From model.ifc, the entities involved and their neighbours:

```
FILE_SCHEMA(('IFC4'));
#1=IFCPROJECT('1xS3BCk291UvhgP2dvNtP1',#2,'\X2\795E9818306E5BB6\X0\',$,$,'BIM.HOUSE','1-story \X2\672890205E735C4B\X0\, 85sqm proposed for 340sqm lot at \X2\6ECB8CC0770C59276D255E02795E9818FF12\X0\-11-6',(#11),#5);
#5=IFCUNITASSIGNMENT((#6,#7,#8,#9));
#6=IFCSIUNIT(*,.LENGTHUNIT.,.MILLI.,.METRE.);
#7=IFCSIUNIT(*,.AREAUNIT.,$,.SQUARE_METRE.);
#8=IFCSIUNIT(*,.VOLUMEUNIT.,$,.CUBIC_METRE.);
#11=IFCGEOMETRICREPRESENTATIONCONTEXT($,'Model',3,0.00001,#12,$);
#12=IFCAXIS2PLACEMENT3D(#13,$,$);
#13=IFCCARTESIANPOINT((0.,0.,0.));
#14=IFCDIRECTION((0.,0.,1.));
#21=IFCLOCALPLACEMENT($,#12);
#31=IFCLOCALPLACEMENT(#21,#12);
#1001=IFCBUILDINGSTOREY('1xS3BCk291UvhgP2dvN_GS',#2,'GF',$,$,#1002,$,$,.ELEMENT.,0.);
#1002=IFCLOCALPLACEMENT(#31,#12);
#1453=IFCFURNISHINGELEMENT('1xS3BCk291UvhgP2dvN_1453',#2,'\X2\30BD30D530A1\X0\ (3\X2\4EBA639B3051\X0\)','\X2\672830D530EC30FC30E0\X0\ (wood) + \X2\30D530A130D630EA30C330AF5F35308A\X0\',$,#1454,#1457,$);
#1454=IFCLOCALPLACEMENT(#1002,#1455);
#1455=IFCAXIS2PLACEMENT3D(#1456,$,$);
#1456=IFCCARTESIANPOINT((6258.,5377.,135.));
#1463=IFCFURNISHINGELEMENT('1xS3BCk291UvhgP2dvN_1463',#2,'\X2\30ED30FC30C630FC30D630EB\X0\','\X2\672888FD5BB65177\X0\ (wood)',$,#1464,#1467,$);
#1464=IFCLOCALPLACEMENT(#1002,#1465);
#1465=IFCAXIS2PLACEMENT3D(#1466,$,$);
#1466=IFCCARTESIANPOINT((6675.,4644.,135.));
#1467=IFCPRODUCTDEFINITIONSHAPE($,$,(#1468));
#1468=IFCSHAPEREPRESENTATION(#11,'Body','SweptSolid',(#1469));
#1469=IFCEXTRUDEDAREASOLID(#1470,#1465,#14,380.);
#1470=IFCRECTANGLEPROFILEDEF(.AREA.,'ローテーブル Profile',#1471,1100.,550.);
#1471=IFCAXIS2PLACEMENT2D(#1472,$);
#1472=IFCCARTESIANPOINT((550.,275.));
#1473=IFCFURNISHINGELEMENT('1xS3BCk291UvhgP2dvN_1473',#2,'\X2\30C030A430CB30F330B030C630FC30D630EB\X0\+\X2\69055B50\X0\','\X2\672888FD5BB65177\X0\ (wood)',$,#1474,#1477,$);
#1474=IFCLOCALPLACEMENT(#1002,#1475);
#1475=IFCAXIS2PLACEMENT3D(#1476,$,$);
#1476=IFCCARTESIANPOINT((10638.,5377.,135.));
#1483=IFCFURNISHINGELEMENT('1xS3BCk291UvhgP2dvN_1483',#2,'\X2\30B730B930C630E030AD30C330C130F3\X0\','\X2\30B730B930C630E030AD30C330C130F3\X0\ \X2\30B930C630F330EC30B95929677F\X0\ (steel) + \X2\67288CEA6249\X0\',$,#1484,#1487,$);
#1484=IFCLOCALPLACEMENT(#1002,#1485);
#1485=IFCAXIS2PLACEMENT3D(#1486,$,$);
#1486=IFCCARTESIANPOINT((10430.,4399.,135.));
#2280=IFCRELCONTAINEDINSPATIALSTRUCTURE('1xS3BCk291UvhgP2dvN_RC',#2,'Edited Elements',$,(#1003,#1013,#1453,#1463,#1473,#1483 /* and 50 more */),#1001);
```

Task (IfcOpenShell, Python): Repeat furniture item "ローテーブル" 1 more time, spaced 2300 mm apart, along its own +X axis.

```python
import ifcopenshell
import ifcopenshell.api.geometry
import ifcopenshell.api.root
import ifcopenshell.util.element
import ifcopenshell.util.placement

model = ifcopenshell.open("model.ifc")


def reuse_history(source, copy):
    """copy_class also copies each property set's owner history, people and application; keep the originals."""
    for rel in copy.IsDefinedBy:
        if rel.is_a("IfcRelDefinesByProperties") and (history := rel.RelatingPropertyDefinition.OwnerHistory):
            rel.RelatingPropertyDefinition.OwnerHistory = source.OwnerHistory
            ifcopenshell.util.element.remove_deep2(model, history)


source = model.by_guid("1xS3BCk291UvhgP2dvN_1463")
base = ifcopenshell.util.placement.get_local_placement(source.ObjectPlacement)
step = base[:3, 0] * 2300.0

for i in range(1, 2):
    copy = ifcopenshell.api.root.copy_class(model, product=source)
    copy.Representation = ifcopenshell.util.element.copy_deep(
        model, source.Representation, exclude=["IfcGeometricRepresentationContext", "IfcRepresentationMap"]
    )
    reuse_history(source, copy)
    matrix = base.copy()
    matrix[:3, 3] += i * step
    print("added at", matrix[:3, 3].round(3) + 0.0)
    ifcopenshell.api.geometry.edit_object_placement(model, product=copy, matrix=matrix, is_si=False)

model.write("model_updated.ifc")
```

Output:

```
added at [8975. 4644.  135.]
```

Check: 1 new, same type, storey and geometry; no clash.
